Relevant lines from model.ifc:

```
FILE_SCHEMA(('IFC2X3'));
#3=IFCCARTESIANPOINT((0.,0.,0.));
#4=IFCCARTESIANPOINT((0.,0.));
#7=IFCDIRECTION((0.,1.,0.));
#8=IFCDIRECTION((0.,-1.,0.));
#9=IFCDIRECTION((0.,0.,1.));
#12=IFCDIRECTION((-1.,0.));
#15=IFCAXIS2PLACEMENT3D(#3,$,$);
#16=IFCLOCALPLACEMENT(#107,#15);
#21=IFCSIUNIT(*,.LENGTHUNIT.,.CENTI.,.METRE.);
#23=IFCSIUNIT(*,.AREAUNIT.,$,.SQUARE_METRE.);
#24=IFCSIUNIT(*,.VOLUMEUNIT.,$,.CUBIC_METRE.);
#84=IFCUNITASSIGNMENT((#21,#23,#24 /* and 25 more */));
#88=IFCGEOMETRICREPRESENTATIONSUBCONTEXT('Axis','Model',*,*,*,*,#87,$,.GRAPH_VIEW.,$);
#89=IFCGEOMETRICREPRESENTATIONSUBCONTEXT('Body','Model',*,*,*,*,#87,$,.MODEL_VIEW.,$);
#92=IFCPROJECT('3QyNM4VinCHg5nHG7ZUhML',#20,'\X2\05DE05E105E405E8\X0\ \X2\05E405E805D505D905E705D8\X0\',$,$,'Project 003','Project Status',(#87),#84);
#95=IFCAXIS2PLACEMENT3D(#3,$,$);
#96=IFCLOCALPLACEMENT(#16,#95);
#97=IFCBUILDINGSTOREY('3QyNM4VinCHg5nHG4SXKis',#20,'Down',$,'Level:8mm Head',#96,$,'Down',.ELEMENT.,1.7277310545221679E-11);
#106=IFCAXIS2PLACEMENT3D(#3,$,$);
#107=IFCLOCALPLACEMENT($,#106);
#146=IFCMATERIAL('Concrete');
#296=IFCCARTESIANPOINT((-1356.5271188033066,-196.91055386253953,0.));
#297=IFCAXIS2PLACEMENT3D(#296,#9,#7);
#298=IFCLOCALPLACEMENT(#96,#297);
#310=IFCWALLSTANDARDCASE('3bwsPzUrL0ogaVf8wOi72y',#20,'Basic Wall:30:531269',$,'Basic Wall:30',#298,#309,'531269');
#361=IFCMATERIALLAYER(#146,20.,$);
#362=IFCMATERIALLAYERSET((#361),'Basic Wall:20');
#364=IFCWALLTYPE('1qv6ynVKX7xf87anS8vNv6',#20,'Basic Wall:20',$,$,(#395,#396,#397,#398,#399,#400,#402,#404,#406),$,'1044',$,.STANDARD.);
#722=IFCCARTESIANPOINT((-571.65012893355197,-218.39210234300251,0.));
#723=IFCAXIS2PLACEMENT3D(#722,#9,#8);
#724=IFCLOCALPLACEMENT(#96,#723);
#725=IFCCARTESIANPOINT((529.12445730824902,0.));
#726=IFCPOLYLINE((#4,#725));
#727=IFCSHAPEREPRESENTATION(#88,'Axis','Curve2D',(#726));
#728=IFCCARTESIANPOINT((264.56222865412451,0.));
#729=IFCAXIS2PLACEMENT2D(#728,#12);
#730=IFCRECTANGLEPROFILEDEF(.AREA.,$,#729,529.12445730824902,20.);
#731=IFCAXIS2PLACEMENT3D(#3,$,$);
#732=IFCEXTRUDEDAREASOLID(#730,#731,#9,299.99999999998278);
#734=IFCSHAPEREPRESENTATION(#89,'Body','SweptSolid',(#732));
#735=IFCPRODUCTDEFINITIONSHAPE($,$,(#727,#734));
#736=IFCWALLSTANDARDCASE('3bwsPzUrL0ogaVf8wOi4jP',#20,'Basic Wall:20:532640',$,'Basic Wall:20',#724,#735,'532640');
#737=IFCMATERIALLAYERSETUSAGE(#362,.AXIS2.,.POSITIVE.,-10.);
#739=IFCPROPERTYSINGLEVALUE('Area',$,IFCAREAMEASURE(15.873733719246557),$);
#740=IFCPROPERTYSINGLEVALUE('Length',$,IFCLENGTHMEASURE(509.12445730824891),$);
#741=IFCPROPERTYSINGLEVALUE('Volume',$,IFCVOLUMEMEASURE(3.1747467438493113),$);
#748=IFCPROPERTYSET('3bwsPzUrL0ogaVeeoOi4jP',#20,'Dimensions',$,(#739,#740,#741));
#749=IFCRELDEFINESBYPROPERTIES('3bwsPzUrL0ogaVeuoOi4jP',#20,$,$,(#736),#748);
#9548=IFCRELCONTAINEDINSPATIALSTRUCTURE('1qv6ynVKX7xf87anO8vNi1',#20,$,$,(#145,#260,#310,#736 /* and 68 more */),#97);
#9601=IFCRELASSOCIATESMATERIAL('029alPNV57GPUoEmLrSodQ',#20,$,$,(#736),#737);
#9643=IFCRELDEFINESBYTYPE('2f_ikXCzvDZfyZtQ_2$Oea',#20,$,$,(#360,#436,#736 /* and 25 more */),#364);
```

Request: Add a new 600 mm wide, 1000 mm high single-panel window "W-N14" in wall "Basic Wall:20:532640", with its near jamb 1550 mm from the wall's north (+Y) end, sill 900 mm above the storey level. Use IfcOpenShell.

```python
import numpy as np
import ifcopenshell
import ifcopenshell.api.feature
import ifcopenshell.api.geometry
import ifcopenshell.api.pset
import ifcopenshell.api.root
import ifcopenshell.api.spatial
import ifcopenshell.api.type
import ifcopenshell.geom
import ifcopenshell.util.element
import ifcopenshell.util.placement
import ifcopenshell.util.representation
import ifcopenshell.util.shape
import ifcopenshell.util.unit

model = ifcopenshell.open("model.ifc")
unit_scale = ifcopenshell.util.unit.calculate_unit_scale(model)
area_scale = ifcopenshell.util.unit.calculate_unit_scale(model, "AREAUNIT")
volume_scale = ifcopenshell.util.unit.calculate_unit_scale(model, "VOLUMEUNIT")
settings = ifcopenshell.geom.settings()


def volume(element):
    """Net volume in cubic metres, openings subtracted."""
    shape = ifcopenshell.geom.create_shape(settings, element)
    return ifcopenshell.util.shape.get_volume(shape.geometry)


wall = model.by_guid("3bwsPzUrL0ogaVf8wOi4jP")
storey = ifcopenshell.util.element.get_container(wall, ifc_class="IfcBuildingStorey")
context = ifcopenshell.util.representation.get_context(model, "Model", "Body", "MODEL_VIEW")
before = volume(wall)

width, height, from_end, sill = 0.6, 1, 1.55, 0.9  # metres

# The wall runs along its own X axis, and the end named is its -X end.
wall_shape = ifcopenshell.geom.create_shape(settings, wall)
x, y, z = ifcopenshell.util.shape.get_vertices(wall_shape.geometry).T
start = x.min() + from_end
face, thickness = float(y.min()), float(y.max() - y.min())
wall_matrix = ifcopenshell.util.placement.get_local_placement(wall.ObjectPlacement)
level = ifcopenshell.util.placement.get_local_placement(storey.ObjectPlacement)[2, 3]


def in_wall(x, y):
    """Placement at x, y metres in the wall's axes, at sill height."""
    matrix = wall_matrix.copy()
    matrix[:, 3] = wall_matrix @ np.array([x / unit_scale, y / unit_scale, 0.0, 1.0])
    matrix[2, 3] = level + sill / unit_scale
    return matrix


# Opening: a box that overshoots both wall faces by 50 mm.
opening = ifcopenshell.api.root.create_entity(model, ifc_class="IfcOpeningElement")
box = ifcopenshell.api.geometry.add_wall_representation(
    model, context=context, length=width, height=height, thickness=thickness + 0.1
)
ifcopenshell.api.geometry.assign_representation(model, product=opening, representation=box)
ifcopenshell.api.geometry.edit_object_placement(model, product=opening, matrix=in_wall(start, face - 0.05), is_si=False)
ifcopenshell.api.feature.add_feature(model, feature=opening, element=wall)

window = ifcopenshell.api.root.create_entity(model, ifc_class="IfcWindow", name="W-N14")
window.OverallWidth, window.OverallHeight = width / unit_scale, height / unit_scale
body = ifcopenshell.api.geometry.add_window_representation(
    model,
    context=context,
    overall_width=window.OverallWidth,
    overall_height=window.OverallHeight,
    partition_type="SINGLE_PANEL",
)
ifcopenshell.api.geometry.assign_representation(model, product=window, representation=body)
ifcopenshell.api.spatial.assign_container(model, products=[window], relating_structure=storey)
fills = ifcopenshell.api.feature.add_filling(model, opening=opening, element=window)
fills.OwnerHistory = window.OwnerHistory  # required in IFC2X3

# IFC2X3 keeps the operation on the window style.
style = ifcopenshell.api.root.create_entity(model, ifc_class="IfcWindowStyle", name="W-N14")
style.OperationType, style.ConstructionType = "SINGLE_PANEL", "NOTDEFINED"
style.ParameterTakesPrecedence = style.Sizeable = False
ifcopenshell.api.type.assign_type(model, related_objects=[window], relating_type=style)

# Centre the window in the wall's thickness.
ifcopenshell.api.geometry.edit_object_placement(model, product=window, matrix=in_wall(start, face), is_si=False)
window_shape = ifcopenshell.geom.create_shape(settings, window)
depth = ifcopenshell.util.shape.get_vertices(window_shape.geometry)[:, 1]
offset = face + thickness / 2 - (depth.min() + depth.max()) / 2
ifcopenshell.api.geometry.edit_object_placement(model, product=window, matrix=in_wall(start, offset), is_si=False)

after = volume(wall)

# Update the wall's stored quantities.
pset = model.by_id(ifcopenshell.util.element.get_pset(wall, "Dimensions", should_inherit=False)["id"])
ifcopenshell.api.pset.edit_pset(model, pset=pset, properties={
    "Area": model.create_entity("IfcAreaMeasure", after / thickness / area_scale),
    "Volume": model.create_entity("IfcVolumeMeasure", after / volume_scale),
})

print(f"wall volume {before:.3f} -> {after:.3f} m3")

model.write("model-out.ifc")
```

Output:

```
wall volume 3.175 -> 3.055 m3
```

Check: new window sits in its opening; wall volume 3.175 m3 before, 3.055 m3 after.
